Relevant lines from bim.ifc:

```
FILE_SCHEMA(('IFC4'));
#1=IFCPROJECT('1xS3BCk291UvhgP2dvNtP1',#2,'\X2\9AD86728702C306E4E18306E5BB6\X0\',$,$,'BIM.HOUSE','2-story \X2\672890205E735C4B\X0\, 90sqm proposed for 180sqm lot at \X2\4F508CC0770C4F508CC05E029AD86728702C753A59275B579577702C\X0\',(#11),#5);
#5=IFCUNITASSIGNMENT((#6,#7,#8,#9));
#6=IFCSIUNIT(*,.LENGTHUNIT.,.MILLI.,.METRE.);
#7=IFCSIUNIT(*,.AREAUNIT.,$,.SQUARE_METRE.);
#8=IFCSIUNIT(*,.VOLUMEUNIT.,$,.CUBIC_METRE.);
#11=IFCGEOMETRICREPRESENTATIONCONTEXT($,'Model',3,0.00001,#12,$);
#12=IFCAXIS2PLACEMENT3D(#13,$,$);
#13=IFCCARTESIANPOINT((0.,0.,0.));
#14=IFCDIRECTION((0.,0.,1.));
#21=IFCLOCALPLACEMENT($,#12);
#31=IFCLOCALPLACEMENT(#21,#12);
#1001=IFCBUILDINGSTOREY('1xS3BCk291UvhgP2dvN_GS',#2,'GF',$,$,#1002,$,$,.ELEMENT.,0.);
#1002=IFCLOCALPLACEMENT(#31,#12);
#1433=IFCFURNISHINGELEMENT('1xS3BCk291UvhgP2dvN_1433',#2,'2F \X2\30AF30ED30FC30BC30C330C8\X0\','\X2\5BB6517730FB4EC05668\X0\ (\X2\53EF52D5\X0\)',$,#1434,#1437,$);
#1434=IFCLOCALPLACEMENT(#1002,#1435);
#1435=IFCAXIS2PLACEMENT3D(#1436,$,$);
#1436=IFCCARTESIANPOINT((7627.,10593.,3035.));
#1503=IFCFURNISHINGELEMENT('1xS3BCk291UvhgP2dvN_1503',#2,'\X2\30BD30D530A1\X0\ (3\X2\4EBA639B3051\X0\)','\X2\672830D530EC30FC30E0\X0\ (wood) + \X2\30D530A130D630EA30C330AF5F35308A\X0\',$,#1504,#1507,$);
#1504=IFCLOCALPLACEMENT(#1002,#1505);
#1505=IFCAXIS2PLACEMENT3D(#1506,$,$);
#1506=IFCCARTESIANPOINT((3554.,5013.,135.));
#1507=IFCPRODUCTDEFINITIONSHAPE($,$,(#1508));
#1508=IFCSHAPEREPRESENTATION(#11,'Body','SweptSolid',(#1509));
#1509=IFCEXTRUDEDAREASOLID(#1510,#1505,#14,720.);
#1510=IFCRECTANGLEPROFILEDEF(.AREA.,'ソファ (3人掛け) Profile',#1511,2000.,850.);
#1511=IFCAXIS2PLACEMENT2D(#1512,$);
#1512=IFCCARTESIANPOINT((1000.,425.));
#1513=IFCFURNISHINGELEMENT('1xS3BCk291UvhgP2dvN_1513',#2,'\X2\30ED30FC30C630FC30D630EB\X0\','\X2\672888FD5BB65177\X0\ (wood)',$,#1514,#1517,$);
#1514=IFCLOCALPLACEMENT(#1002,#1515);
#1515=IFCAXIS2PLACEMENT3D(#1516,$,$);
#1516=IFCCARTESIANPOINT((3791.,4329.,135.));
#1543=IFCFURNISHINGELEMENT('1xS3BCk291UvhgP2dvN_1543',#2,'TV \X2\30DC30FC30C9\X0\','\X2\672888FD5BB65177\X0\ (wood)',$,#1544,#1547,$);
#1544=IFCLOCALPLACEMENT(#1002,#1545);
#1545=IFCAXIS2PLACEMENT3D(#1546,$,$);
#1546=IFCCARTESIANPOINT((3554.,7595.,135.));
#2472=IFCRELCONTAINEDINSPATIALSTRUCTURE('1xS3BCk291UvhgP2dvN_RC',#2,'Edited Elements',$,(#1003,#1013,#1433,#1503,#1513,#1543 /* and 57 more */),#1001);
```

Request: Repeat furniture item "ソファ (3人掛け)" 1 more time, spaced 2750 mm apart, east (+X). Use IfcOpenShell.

```python
import numpy as np
import ifcopenshell
import ifcopenshell.api.geometry
import ifcopenshell.api.root
import ifcopenshell.util.element
import ifcopenshell.util.placement
import ifcopenshell.util.unit

model = ifcopenshell.open("bim.ifc")
unit_scale = ifcopenshell.util.unit.calculate_unit_scale(model)


def reuse_history(source, copy):
    """copy_class also copies each property set's owner history, people and application; keep the originals."""
    for rel in copy.IsDefinedBy:
        if rel.is_a("IfcRelDefinesByProperties") and (history := rel.RelatingPropertyDefinition.OwnerHistory):
            rel.RelatingPropertyDefinition.OwnerHistory = source.OwnerHistory
            ifcopenshell.util.element.remove_deep2(model, history)


source = model.by_guid("1xS3BCk291UvhgP2dvN_1503")
base = ifcopenshell.util.placement.get_local_placement(source.ObjectPlacement)
step = np.array([1.0, 0.0, 0.0]) * 2.75 / unit_scale

for i in range(1, 2):
    copy = ifcopenshell.api.root.copy_class(model, product=source)
    copy.Representation = ifcopenshell.util.element.copy_deep(
        model, source.Representation, exclude=["IfcGeometricRepresentationContext", "IfcRepresentationMap"]
    )
    reuse_history(source, copy)
    matrix = base.copy()
    matrix[:3, 3] += i * step
    print("added at", matrix[:3, 3].round(3) + 0.0)
    ifcopenshell.api.geometry.edit_object_placement(model, product=copy, matrix=matrix, is_si=False)

model.write("bim_edited.ifc")
```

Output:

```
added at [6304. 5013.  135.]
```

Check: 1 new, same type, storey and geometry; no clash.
